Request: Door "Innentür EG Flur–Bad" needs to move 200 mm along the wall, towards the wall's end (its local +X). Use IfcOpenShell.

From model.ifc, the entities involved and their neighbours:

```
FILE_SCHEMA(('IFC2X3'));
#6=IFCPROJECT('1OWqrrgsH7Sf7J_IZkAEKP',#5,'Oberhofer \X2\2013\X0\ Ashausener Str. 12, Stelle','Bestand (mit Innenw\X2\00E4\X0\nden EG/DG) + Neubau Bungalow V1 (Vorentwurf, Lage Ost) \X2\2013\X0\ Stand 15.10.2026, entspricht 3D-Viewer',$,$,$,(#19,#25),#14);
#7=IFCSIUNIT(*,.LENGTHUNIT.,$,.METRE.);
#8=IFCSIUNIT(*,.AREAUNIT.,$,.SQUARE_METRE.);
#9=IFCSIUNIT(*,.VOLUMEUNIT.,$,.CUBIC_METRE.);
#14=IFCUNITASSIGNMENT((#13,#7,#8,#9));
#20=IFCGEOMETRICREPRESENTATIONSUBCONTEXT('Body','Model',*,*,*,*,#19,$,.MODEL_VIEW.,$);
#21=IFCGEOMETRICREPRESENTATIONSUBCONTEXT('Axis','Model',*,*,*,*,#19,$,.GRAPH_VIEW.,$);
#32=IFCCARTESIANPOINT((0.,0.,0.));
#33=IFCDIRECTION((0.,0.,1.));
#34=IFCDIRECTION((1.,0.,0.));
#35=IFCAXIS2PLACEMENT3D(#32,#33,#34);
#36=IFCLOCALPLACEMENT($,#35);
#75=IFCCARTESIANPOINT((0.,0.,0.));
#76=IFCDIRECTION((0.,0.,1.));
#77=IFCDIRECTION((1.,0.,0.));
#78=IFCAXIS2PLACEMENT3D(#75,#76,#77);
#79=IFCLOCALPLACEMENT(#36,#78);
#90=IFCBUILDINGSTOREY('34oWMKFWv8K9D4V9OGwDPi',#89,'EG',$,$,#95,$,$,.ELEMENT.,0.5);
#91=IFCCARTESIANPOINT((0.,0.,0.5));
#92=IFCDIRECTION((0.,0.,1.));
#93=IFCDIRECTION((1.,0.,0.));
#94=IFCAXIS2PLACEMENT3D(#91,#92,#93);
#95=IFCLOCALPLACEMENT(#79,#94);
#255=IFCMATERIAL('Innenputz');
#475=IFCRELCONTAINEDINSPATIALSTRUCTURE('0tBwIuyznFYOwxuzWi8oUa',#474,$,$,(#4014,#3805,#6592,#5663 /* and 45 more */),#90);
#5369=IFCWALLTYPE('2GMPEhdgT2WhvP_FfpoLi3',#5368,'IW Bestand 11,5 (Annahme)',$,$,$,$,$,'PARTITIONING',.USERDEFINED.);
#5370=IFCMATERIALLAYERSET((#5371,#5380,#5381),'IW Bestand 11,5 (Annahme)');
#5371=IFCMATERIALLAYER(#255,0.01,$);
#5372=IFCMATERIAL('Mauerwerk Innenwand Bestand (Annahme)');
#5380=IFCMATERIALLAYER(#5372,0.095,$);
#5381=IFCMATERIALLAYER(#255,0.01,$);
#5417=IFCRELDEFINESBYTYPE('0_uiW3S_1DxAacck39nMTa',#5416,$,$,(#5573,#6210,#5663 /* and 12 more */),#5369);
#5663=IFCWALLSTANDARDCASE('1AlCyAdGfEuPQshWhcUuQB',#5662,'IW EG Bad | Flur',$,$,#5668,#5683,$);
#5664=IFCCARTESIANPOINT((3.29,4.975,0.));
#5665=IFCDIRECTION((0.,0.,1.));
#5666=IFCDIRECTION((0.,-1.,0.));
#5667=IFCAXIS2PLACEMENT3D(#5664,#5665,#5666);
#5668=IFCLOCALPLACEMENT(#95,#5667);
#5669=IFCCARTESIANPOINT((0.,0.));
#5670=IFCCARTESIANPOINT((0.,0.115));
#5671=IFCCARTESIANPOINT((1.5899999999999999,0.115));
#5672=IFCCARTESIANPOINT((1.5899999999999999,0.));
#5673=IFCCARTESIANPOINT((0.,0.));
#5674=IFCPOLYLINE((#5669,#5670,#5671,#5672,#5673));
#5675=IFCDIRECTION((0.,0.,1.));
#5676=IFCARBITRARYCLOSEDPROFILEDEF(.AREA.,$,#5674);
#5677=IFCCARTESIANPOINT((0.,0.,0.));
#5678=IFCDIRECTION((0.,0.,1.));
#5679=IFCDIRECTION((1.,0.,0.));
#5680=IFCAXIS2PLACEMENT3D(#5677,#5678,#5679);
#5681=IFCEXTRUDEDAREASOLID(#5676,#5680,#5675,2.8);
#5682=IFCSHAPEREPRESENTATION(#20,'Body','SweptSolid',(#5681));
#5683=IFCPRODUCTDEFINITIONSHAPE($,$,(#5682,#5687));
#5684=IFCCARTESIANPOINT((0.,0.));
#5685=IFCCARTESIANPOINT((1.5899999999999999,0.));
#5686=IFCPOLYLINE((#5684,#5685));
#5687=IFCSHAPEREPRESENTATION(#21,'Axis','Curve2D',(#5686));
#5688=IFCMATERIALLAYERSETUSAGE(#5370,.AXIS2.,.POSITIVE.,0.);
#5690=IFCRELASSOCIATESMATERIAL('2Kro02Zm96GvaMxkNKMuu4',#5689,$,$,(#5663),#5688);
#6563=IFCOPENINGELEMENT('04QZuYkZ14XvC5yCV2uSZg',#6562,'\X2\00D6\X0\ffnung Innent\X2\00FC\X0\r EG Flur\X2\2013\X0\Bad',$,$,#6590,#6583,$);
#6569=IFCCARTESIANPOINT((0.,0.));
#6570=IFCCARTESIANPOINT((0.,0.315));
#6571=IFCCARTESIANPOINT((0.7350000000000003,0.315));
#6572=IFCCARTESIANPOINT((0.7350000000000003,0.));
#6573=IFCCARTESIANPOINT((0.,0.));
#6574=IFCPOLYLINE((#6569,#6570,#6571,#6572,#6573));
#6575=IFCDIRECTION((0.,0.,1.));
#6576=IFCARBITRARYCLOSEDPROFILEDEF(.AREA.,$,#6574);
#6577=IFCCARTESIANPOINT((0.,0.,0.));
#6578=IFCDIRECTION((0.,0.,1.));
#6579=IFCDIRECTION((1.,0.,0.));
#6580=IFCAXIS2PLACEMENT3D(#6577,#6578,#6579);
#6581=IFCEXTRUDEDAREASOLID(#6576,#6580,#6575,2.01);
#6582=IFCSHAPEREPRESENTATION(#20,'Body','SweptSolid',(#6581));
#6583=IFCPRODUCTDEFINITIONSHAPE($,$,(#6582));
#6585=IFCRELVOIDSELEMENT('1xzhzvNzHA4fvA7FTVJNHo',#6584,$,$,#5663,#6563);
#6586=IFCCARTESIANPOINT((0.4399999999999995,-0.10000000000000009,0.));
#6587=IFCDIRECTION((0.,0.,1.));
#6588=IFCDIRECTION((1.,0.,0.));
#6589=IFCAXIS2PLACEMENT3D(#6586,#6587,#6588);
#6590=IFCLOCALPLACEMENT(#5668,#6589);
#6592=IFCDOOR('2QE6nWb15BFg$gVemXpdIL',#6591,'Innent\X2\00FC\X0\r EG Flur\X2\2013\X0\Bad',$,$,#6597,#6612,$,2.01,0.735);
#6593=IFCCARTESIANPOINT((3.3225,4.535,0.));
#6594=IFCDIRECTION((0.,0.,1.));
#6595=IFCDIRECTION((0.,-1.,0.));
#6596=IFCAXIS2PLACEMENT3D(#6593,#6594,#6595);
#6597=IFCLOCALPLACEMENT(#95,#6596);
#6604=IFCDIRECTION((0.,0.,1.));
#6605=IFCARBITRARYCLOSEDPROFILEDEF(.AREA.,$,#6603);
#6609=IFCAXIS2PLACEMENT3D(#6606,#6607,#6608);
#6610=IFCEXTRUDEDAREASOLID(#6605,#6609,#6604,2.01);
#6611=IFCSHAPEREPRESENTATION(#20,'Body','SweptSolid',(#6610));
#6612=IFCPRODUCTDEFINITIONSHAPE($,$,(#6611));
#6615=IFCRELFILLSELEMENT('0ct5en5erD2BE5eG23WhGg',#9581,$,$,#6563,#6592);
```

```python
import ifcopenshell
import ifcopenshell.api.geometry
import ifcopenshell.util.placement

model = ifcopenshell.open("model.ifc")

door = model.by_id(6592)
opening = door.FillsVoids[0].RelatingOpeningElement
wall = opening.VoidsElements[0].RelatingBuildingElement

wall_matrix = ifcopenshell.util.placement.get_local_placement(wall.ObjectPlacement)
shift = wall_matrix[:3, 0] * 0.2
before = ifcopenshell.util.placement.get_local_placement(door.ObjectPlacement)[:3, 3].copy()

# The door is not placed relative to its opening, so move both.
for product in (opening, door):
    matrix = ifcopenshell.util.placement.get_local_placement(product.ObjectPlacement)
    matrix[:3, 3] += shift
    ifcopenshell.api.geometry.edit_object_placement(model, product=product, matrix=matrix, is_si=False)

after = ifcopenshell.util.placement.get_local_placement(door.ObjectPlacement)[:3, 3]
print("door moved by", (after - before).round(3) + 0.0)

model.write("model-out.ifc")
```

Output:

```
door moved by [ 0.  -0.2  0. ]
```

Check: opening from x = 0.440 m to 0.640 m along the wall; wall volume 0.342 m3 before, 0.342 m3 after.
